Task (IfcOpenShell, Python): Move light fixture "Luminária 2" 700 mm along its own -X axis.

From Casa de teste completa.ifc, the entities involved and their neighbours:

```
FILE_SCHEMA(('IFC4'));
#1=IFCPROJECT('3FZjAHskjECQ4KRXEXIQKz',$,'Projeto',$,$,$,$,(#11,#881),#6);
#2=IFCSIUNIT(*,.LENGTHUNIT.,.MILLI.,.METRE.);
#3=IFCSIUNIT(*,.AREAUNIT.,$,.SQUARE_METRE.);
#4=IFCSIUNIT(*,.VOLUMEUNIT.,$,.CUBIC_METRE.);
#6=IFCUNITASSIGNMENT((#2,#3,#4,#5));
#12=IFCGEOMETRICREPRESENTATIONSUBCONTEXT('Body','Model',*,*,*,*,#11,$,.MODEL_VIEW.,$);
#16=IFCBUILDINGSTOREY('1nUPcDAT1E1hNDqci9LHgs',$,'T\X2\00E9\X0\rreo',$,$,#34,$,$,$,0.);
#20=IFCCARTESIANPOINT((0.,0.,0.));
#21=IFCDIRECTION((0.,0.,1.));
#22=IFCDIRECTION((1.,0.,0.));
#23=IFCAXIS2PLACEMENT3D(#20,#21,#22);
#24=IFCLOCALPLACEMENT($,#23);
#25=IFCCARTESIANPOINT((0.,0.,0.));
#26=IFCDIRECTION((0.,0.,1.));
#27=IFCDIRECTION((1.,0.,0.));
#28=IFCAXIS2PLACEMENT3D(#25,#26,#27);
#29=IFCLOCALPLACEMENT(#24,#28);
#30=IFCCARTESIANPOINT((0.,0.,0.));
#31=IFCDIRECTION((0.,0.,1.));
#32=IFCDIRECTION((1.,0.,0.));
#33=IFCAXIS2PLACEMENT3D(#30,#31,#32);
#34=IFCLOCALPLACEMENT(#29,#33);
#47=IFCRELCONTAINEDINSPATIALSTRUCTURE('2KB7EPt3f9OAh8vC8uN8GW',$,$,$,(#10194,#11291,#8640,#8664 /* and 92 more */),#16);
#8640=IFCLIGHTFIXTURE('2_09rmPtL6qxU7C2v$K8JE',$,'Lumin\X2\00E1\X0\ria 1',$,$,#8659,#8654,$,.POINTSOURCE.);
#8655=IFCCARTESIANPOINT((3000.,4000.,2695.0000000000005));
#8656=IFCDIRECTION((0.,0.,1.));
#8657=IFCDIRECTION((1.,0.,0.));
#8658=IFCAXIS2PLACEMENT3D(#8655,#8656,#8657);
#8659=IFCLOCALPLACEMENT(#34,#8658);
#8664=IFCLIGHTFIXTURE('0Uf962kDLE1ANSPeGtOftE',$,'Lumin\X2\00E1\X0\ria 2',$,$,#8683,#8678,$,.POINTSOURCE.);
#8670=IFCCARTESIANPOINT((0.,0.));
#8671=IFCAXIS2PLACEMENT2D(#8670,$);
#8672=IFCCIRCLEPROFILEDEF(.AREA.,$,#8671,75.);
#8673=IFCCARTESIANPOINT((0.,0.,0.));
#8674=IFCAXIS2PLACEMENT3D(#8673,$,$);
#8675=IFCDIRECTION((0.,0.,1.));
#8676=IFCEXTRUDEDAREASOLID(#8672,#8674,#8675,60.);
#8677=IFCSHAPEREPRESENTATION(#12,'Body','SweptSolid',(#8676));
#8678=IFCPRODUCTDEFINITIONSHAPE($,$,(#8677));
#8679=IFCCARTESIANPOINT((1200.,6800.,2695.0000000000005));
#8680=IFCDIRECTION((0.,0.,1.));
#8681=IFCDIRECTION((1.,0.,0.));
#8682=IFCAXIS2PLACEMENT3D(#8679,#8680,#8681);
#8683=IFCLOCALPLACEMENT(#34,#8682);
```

```python
import ifcopenshell
import ifcopenshell.api.geometry
import ifcopenshell.util.placement

model = ifcopenshell.open("Casa de teste completa.ifc")

item = model.by_guid("0Uf962kDLE1ANSPeGtOftE")
matrix = ifcopenshell.util.placement.get_local_placement(item.ObjectPlacement)
matrix[:3, 3] -= matrix[:3, 0] * 700.0
ifcopenshell.api.geometry.edit_object_placement(model, product=item, matrix=matrix, is_si=False)

print(ifcopenshell.util.placement.get_local_placement(item.ObjectPlacement).round(3) + 0.0)

model.write("Casa de teste completa_updated.ifc")
```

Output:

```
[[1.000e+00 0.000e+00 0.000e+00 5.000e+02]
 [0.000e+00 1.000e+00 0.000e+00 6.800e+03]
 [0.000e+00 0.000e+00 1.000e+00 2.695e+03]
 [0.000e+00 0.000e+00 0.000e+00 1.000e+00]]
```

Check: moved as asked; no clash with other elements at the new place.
